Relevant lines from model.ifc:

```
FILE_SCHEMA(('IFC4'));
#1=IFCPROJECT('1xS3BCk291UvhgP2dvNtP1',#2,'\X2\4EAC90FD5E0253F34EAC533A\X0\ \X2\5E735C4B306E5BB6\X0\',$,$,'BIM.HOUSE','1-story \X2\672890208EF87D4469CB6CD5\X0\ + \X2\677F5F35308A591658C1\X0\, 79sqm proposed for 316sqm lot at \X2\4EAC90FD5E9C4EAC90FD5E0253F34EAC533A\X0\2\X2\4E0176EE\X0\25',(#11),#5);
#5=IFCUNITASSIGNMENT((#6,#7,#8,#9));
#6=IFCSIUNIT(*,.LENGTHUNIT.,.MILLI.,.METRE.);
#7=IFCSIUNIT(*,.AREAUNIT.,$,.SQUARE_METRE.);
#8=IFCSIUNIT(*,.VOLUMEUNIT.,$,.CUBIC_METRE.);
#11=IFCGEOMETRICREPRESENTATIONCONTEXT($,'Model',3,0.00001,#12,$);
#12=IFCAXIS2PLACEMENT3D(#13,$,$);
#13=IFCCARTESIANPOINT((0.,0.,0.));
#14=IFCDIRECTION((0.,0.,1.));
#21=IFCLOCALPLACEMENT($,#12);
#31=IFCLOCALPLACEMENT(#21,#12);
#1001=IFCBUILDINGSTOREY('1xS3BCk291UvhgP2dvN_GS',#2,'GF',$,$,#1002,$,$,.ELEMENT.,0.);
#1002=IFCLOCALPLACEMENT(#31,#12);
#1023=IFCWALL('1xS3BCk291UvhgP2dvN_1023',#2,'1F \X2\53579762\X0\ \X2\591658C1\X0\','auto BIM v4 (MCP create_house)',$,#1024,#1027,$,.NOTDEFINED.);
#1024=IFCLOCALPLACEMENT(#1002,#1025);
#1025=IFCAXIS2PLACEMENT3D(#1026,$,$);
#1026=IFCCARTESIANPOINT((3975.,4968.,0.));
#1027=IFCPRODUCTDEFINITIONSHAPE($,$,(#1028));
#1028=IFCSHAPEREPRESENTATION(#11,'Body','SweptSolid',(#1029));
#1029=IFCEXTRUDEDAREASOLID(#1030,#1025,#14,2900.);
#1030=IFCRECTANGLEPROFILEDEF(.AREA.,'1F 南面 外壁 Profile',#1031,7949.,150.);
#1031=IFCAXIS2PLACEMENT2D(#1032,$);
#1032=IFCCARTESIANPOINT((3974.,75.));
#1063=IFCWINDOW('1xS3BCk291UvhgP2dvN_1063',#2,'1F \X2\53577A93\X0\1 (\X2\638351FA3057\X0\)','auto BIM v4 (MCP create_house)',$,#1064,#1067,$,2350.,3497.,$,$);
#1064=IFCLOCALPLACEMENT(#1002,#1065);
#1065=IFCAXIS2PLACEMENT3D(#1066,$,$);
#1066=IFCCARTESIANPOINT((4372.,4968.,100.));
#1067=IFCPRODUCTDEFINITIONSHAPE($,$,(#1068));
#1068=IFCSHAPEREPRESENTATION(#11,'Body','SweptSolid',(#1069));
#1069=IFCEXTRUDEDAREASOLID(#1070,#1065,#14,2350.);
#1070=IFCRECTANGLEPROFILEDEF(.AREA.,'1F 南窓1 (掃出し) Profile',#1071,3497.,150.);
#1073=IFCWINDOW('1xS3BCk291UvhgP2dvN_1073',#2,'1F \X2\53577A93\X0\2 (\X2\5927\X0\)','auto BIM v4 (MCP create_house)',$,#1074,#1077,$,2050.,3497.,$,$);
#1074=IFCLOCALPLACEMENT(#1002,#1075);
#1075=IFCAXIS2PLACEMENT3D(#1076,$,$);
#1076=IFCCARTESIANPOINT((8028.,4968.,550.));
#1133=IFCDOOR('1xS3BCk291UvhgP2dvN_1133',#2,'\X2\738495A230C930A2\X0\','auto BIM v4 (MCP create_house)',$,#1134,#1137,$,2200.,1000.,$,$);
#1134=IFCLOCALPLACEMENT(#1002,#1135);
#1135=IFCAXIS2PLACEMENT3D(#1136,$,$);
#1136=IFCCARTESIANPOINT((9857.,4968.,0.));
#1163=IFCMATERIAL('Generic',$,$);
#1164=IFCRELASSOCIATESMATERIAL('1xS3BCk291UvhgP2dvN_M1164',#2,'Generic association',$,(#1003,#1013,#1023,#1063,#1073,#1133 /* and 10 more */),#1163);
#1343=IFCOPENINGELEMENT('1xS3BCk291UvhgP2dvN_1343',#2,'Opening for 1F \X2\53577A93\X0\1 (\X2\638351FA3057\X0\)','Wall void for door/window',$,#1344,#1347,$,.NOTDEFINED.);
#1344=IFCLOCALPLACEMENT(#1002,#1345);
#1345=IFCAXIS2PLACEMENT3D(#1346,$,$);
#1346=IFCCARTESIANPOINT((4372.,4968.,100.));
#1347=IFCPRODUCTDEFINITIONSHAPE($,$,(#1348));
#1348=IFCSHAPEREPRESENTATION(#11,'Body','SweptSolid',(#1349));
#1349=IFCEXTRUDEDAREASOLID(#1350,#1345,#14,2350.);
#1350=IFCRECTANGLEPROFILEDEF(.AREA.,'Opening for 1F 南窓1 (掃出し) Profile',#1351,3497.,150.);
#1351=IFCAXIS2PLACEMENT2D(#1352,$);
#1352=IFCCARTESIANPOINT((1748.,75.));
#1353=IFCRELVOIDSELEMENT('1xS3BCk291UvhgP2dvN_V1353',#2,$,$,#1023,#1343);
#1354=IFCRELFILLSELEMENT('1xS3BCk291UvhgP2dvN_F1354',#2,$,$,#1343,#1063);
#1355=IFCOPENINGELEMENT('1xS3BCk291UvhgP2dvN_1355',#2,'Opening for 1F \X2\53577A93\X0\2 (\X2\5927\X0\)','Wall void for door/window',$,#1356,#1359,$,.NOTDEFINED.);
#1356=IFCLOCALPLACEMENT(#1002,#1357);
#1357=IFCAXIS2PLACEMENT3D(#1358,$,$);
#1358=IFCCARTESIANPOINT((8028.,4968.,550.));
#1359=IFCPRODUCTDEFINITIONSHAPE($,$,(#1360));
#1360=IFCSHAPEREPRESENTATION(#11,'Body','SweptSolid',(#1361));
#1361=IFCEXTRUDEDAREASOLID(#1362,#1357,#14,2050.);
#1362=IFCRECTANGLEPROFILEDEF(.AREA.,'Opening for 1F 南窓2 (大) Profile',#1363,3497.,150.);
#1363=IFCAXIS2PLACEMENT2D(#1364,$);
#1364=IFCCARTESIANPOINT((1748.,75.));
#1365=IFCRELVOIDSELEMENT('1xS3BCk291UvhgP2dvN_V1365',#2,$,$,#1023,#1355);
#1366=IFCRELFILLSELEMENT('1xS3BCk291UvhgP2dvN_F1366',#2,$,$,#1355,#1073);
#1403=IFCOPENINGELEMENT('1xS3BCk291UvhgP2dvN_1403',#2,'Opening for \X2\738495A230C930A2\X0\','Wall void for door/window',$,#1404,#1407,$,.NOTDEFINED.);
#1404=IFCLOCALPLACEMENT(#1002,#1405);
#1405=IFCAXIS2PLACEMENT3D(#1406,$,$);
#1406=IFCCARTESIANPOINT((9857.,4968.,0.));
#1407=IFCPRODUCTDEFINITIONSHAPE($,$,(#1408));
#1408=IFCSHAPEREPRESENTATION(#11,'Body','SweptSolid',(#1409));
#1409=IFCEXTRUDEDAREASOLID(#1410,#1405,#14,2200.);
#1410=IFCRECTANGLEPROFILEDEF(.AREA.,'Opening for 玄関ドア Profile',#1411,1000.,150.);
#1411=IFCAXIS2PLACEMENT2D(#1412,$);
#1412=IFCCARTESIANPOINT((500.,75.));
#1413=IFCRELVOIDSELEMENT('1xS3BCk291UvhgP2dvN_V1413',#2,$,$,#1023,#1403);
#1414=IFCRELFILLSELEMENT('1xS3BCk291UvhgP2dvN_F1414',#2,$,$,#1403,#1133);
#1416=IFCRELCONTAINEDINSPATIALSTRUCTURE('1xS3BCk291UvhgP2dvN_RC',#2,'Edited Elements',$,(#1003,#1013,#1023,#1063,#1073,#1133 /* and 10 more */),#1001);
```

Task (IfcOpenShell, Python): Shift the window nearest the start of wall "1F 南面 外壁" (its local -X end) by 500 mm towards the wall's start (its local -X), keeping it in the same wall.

```python
import ifcopenshell
import ifcopenshell.api.geometry
import ifcopenshell.util.placement

model = ifcopenshell.open("model.ifc")

window = model.by_guid("1xS3BCk291UvhgP2dvN_1063")
opening = window.FillsVoids[0].RelatingOpeningElement
wall = opening.VoidsElements[0].RelatingBuildingElement

wall_matrix = ifcopenshell.util.placement.get_local_placement(wall.ObjectPlacement)
shift = wall_matrix[:3, 0] * -500.0
before = ifcopenshell.util.placement.get_local_placement(window.ObjectPlacement)[:3, 3].copy()

# The window is not placed relative to its opening, so move both.
for product in (opening, window):
    matrix = ifcopenshell.util.placement.get_local_placement(product.ObjectPlacement)
    matrix[:3, 3] += shift
    ifcopenshell.api.geometry.edit_object_placement(model, product=product, matrix=matrix, is_si=False)

after = ifcopenshell.util.placement.get_local_placement(window.ObjectPlacement)[:3, 3]
print("window moved by", (after - before).round(3) + 0.0)

model.write("model-out.ifc")
```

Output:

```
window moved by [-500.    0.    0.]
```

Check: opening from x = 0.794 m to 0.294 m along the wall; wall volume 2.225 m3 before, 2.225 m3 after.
